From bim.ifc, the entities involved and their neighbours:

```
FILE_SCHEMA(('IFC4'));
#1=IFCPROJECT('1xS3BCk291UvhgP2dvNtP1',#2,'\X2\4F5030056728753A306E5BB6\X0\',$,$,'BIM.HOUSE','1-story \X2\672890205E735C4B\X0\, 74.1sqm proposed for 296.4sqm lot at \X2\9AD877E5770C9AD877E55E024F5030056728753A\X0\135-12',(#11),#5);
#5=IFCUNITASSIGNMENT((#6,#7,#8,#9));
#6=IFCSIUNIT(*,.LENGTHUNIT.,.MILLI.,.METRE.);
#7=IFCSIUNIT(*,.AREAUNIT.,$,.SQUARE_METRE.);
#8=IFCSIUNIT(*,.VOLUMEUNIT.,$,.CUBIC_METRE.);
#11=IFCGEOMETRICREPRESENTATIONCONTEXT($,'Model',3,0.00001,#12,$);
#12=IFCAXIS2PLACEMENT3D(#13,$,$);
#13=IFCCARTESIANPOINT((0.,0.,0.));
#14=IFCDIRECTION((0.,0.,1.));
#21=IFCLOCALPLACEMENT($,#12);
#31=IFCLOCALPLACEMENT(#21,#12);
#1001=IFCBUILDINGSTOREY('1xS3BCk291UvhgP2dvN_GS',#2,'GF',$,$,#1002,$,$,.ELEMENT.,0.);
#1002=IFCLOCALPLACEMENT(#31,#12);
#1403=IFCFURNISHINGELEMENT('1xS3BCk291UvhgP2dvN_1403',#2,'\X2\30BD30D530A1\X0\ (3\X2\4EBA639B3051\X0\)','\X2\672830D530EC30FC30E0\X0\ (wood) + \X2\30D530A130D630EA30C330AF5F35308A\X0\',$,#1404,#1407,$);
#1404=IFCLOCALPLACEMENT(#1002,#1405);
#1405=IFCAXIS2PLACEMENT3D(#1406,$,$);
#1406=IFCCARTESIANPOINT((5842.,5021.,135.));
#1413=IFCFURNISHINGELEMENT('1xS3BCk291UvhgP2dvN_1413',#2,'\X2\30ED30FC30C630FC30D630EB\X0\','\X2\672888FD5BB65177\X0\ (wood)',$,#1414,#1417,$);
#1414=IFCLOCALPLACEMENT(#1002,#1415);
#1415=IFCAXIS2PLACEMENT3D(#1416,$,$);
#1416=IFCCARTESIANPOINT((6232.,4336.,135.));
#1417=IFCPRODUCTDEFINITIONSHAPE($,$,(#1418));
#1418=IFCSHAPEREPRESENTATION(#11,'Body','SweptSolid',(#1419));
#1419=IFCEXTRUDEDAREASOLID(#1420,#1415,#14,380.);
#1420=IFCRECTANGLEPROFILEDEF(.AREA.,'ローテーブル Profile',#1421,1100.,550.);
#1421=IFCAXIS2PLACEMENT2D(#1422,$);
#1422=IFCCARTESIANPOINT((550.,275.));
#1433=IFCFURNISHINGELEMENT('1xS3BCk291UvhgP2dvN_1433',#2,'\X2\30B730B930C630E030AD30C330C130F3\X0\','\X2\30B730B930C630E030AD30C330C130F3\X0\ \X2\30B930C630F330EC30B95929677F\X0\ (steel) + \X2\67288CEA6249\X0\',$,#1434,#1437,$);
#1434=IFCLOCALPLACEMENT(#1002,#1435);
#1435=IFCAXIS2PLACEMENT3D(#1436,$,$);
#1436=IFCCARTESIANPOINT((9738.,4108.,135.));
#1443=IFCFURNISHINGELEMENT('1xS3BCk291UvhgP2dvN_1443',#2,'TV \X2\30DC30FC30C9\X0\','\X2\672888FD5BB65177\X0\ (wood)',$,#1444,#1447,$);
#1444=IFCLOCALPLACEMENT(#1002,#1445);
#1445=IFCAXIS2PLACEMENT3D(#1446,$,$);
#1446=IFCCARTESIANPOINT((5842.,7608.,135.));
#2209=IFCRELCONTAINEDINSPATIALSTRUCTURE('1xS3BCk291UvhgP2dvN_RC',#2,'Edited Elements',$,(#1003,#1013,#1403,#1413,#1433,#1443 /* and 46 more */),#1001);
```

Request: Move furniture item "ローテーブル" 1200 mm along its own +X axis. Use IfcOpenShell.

```python
import ifcopenshell
import ifcopenshell.api.geometry
import ifcopenshell.util.placement
import ifcopenshell.util.unit

model = ifcopenshell.open("bim.ifc")
unit_scale = ifcopenshell.util.unit.calculate_unit_scale(model)

item = model.by_guid("1xS3BCk291UvhgP2dvN_1413")
matrix = ifcopenshell.util.placement.get_local_placement(item.ObjectPlacement)
matrix[:3, 3] += matrix[:3, 0] * 1.2 / unit_scale
ifcopenshell.api.geometry.edit_object_placement(model, product=item, matrix=matrix, is_si=False)

print(ifcopenshell.util.placement.get_local_placement(item.ObjectPlacement).round(3) + 0.0)

model.write("bim-out.ifc")
```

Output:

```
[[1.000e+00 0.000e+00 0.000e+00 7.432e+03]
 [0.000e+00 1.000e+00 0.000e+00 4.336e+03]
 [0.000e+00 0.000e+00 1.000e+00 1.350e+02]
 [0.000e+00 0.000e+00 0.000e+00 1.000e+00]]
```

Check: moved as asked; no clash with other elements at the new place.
